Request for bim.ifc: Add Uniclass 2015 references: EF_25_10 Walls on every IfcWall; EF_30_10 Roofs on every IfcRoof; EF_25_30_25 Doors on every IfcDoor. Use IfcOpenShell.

First a look at what the model holds.

```python
import ifcopenshell

model = ifcopenshell.open("bim.ifc")
print(model.schema)
print("classifications:", [c.Name for c in model.by_type("IfcClassification")])
for ifc_class in ("IfcDoor", "IfcRoof", "IfcStair", "IfcWall", "IfcWindow"):
    print(ifc_class, len(model.by_type(ifc_class)))
```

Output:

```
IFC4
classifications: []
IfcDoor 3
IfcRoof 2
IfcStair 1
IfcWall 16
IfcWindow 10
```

```python
import ifcopenshell
import ifcopenshell.api.classification

model = ifcopenshell.open("bim.ifc")

system = ifcopenshell.api.classification.add_classification(model, classification="Uniclass 2015")

codes = {
    "IfcWall": ("EF_25_10", "Walls"),
    "IfcRoof": ("EF_30_10", "Roofs"),
    "IfcDoor": ("EF_25_30_25", "Doors"),
}
for ifc_class, (code, name) in codes.items():
    products = model.by_type(ifc_class)
    ifcopenshell.api.classification.add_reference(
        model, products=products, classification=system, identification=code, name=name
    )
    print(code, len(products))

model.write("bim_updated.ifc")
```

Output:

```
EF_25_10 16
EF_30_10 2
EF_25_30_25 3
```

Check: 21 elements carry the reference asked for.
